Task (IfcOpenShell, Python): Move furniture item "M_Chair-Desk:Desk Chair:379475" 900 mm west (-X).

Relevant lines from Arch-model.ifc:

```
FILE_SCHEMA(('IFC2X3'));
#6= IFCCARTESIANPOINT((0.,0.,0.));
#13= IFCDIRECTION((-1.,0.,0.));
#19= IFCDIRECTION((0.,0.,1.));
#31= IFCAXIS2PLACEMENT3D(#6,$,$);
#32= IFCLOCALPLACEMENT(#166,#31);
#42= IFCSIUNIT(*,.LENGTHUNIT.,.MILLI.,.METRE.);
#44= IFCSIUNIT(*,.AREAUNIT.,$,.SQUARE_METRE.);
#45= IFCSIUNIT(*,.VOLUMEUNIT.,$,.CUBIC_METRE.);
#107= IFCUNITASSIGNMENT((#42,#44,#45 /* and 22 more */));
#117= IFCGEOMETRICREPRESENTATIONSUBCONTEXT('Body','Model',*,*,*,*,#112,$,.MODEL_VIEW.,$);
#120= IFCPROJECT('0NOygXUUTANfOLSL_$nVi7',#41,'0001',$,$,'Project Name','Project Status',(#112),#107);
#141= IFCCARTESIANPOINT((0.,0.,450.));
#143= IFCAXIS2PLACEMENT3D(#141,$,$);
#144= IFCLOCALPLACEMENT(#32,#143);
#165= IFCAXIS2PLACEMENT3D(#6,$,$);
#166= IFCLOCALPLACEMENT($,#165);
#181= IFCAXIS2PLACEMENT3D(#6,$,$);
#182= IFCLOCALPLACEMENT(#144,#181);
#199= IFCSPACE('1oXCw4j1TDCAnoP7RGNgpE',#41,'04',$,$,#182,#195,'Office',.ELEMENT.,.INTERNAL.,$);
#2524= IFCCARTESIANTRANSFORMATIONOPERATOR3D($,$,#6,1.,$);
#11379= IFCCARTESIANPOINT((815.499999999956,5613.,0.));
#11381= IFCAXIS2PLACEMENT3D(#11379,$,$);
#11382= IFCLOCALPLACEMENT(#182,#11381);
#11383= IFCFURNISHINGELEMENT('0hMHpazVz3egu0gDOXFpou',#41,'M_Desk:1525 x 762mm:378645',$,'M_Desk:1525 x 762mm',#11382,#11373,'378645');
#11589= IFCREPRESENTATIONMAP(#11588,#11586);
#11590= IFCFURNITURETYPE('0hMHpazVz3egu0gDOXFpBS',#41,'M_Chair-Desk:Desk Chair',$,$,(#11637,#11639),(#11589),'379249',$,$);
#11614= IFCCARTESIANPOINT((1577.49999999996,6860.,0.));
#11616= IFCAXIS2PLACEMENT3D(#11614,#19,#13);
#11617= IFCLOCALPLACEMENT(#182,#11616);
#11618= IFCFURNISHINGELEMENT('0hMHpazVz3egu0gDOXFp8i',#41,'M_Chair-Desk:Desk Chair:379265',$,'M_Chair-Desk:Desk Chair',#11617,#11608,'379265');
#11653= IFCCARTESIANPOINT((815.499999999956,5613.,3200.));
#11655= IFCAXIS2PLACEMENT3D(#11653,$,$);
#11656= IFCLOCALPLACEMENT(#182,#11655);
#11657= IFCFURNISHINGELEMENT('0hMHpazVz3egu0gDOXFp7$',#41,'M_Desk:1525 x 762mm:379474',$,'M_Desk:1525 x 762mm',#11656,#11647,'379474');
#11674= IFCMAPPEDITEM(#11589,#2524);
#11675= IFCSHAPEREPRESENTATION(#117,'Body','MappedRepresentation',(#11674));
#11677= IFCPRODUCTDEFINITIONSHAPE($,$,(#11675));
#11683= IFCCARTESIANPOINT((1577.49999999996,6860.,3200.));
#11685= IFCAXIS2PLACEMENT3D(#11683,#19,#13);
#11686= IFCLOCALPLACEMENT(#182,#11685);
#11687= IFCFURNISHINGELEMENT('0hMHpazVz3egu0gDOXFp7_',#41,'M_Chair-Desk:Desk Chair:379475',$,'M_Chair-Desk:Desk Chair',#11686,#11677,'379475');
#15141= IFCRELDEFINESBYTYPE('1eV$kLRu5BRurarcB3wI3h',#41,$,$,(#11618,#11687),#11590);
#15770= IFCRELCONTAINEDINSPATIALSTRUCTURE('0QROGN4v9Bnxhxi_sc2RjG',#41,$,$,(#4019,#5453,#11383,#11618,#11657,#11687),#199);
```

```python
import ifcopenshell
import ifcopenshell.api.geometry
import ifcopenshell.util.placement

model = ifcopenshell.open("Arch-model.ifc")

item = model.by_guid("0hMHpazVz3egu0gDOXFp7_")
matrix = ifcopenshell.util.placement.get_local_placement(item.ObjectPlacement)
matrix[0, 3] -= 900.0
ifcopenshell.api.geometry.edit_object_placement(model, product=item, matrix=matrix, is_si=False)

print(ifcopenshell.util.placement.get_local_placement(item.ObjectPlacement).round(3) + 0.0)

model.write("Arch-model_v2.ifc")
```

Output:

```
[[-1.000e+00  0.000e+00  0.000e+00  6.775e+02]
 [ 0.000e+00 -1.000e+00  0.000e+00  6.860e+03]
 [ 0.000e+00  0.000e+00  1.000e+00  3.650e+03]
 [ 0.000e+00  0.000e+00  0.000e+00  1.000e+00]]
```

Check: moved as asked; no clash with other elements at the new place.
